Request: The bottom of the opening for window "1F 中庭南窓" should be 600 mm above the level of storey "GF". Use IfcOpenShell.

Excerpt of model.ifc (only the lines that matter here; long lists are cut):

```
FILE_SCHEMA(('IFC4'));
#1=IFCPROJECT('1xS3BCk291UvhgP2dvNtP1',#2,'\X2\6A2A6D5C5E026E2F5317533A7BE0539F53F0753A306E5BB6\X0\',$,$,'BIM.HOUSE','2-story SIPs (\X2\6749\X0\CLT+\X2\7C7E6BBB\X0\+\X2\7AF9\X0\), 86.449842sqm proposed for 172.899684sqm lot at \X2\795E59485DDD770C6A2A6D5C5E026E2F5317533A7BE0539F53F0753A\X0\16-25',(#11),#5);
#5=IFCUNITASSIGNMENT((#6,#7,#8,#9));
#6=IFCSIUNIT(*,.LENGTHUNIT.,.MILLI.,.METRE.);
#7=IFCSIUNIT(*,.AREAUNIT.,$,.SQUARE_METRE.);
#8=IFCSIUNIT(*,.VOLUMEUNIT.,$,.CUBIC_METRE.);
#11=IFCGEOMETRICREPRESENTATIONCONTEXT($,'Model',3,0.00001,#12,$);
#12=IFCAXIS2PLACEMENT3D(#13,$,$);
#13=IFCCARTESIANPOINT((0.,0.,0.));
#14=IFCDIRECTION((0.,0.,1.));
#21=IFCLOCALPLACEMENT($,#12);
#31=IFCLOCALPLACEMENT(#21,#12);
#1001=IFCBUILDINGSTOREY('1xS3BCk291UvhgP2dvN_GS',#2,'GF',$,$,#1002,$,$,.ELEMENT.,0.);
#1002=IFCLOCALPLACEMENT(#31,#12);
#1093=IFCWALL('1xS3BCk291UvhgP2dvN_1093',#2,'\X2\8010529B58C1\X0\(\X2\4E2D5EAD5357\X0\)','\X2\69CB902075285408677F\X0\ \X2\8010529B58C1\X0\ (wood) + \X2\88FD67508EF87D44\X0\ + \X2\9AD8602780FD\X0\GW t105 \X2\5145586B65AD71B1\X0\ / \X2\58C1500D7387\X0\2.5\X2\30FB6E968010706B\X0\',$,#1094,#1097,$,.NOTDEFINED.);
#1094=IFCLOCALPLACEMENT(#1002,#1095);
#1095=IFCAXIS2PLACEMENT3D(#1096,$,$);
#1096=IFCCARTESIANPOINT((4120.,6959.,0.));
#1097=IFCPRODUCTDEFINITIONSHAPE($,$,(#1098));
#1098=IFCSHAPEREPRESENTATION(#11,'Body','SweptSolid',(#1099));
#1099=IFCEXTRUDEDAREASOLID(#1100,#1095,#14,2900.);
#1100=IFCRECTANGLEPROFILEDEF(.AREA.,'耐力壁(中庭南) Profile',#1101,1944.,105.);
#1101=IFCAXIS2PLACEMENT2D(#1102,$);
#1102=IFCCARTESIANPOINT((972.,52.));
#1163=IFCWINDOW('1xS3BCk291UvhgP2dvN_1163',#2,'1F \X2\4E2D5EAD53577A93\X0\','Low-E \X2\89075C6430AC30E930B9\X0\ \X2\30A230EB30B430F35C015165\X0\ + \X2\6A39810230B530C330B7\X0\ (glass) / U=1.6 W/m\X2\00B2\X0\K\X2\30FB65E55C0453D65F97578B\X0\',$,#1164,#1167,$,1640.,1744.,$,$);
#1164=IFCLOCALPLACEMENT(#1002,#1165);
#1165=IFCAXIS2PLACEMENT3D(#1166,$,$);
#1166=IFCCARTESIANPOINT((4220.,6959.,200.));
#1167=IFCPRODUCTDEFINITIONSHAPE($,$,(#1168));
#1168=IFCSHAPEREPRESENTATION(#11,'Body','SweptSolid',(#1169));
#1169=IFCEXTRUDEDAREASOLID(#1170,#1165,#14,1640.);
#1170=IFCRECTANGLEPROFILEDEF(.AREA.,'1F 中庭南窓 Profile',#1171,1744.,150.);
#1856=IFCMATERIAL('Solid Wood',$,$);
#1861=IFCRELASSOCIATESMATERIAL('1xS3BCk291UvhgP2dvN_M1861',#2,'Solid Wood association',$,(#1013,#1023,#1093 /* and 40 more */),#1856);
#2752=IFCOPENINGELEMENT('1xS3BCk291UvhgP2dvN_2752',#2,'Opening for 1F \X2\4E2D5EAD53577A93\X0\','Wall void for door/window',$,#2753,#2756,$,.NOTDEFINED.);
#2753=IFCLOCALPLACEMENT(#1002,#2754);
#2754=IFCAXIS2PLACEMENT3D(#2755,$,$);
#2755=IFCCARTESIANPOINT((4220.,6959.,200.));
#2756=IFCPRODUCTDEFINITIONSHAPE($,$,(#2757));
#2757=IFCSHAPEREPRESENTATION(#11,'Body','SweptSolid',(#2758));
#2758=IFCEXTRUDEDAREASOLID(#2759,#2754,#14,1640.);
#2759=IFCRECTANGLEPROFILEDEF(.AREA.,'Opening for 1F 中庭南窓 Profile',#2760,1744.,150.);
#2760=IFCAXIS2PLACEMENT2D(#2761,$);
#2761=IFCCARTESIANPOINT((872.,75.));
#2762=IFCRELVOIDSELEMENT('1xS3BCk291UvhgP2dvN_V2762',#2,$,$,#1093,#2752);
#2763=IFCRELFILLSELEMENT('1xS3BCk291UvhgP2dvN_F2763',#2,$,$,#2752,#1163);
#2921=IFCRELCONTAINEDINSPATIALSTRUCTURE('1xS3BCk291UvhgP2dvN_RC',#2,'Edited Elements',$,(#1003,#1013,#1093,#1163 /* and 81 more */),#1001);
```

```python
import numpy as np
import ifcopenshell
import ifcopenshell.api.geometry
import ifcopenshell.geom
import ifcopenshell.util.element
import ifcopenshell.util.placement
import ifcopenshell.util.shape
import ifcopenshell.util.unit

model = ifcopenshell.open("model.ifc")
unit_scale = ifcopenshell.util.unit.calculate_unit_scale(model)

window = model.by_guid("1xS3BCk291UvhgP2dvN_1163")
opening = window.FillsVoids[0].RelatingOpeningElement
storey = ifcopenshell.util.element.get_container(window, ifc_class="IfcBuildingStorey")
level = ifcopenshell.util.placement.get_local_placement(storey.ObjectPlacement)[2, 3]

# The opening's origin need not be at the sill, so measure its lowest point.
shape = ifcopenshell.geom.create_shape(ifcopenshell.geom.settings(), opening)
bottom = ifcopenshell.util.shape.get_shape_bottom_elevation(shape, shape.geometry) / unit_scale
dz = level + 0.6 / unit_scale - bottom

shift = np.array([0.0, 0.0, dz])
# The window is not placed relative to its opening, so move both.
for product in (opening, window):
    matrix = ifcopenshell.util.placement.get_local_placement(product.ObjectPlacement)
    matrix[:3, 3] += shift
    ifcopenshell.api.geometry.edit_object_placement(model, product=product, matrix=matrix, is_si=False)

print(f"moved by {dz * unit_scale:+.3f} m")

model.write("model_rev.ifc")
```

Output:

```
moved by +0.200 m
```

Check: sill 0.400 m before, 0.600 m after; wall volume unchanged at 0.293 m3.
